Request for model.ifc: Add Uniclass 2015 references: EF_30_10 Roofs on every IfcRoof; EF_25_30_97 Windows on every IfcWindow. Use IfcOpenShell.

First a look at what the model holds.

```python
import ifcopenshell

model = ifcopenshell.open("model.ifc")
print(model.schema)
print("classifications:", [c.Name for c in model.by_type("IfcClassification")])
for ifc_class in ("IfcDoor", "IfcRoof", "IfcStair", "IfcWall", "IfcWindow"):
    print(ifc_class, len(model.by_type(ifc_class)))
```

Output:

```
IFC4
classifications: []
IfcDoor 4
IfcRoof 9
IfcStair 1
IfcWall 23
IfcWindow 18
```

```python
import ifcopenshell
import ifcopenshell.api.classification

model = ifcopenshell.open("model.ifc")

system = ifcopenshell.api.classification.add_classification(model, classification="Uniclass 2015")

codes = {
    "IfcRoof": ("EF_30_10", "Roofs"),
    "IfcWindow": ("EF_25_30_97", "Windows"),
}
for ifc_class, (code, name) in codes.items():
    products = model.by_type(ifc_class)
    ifcopenshell.api.classification.add_reference(
        model, products=products, classification=system, identification=code, name=name
    )
    print(code, len(products))

model.write("model_edited.ifc")
```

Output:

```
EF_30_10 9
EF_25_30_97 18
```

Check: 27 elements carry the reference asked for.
